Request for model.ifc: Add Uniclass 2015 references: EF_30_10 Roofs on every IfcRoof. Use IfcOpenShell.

First a look at what the model holds.

```python
import ifcopenshell

model = ifcopenshell.open("model.ifc")
print(model.schema)
print("classifications:", [c.Name for c in model.by_type("IfcClassification")])
for ifc_class in ("IfcDoor", "IfcRoof", "IfcStair", "IfcWall", "IfcWindow"):
    print(ifc_class, len(model.by_type(ifc_class)))
```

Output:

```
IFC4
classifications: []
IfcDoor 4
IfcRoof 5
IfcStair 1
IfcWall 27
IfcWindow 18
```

```python
import ifcopenshell
import ifcopenshell.api.classification

model = ifcopenshell.open("model.ifc")

system = ifcopenshell.api.classification.add_classification(model, classification="Uniclass 2015")

codes = {
    "IfcRoof": ("EF_30_10", "Roofs"),
}
for ifc_class, (code, name) in codes.items():
    products = model.by_type(ifc_class)
    ifcopenshell.api.classification.add_reference(
        model, products=products, classification=system, identification=code, name=name
    )
    print(code, len(products))

model.write("model_rev.ifc")
```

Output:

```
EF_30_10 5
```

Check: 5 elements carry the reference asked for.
